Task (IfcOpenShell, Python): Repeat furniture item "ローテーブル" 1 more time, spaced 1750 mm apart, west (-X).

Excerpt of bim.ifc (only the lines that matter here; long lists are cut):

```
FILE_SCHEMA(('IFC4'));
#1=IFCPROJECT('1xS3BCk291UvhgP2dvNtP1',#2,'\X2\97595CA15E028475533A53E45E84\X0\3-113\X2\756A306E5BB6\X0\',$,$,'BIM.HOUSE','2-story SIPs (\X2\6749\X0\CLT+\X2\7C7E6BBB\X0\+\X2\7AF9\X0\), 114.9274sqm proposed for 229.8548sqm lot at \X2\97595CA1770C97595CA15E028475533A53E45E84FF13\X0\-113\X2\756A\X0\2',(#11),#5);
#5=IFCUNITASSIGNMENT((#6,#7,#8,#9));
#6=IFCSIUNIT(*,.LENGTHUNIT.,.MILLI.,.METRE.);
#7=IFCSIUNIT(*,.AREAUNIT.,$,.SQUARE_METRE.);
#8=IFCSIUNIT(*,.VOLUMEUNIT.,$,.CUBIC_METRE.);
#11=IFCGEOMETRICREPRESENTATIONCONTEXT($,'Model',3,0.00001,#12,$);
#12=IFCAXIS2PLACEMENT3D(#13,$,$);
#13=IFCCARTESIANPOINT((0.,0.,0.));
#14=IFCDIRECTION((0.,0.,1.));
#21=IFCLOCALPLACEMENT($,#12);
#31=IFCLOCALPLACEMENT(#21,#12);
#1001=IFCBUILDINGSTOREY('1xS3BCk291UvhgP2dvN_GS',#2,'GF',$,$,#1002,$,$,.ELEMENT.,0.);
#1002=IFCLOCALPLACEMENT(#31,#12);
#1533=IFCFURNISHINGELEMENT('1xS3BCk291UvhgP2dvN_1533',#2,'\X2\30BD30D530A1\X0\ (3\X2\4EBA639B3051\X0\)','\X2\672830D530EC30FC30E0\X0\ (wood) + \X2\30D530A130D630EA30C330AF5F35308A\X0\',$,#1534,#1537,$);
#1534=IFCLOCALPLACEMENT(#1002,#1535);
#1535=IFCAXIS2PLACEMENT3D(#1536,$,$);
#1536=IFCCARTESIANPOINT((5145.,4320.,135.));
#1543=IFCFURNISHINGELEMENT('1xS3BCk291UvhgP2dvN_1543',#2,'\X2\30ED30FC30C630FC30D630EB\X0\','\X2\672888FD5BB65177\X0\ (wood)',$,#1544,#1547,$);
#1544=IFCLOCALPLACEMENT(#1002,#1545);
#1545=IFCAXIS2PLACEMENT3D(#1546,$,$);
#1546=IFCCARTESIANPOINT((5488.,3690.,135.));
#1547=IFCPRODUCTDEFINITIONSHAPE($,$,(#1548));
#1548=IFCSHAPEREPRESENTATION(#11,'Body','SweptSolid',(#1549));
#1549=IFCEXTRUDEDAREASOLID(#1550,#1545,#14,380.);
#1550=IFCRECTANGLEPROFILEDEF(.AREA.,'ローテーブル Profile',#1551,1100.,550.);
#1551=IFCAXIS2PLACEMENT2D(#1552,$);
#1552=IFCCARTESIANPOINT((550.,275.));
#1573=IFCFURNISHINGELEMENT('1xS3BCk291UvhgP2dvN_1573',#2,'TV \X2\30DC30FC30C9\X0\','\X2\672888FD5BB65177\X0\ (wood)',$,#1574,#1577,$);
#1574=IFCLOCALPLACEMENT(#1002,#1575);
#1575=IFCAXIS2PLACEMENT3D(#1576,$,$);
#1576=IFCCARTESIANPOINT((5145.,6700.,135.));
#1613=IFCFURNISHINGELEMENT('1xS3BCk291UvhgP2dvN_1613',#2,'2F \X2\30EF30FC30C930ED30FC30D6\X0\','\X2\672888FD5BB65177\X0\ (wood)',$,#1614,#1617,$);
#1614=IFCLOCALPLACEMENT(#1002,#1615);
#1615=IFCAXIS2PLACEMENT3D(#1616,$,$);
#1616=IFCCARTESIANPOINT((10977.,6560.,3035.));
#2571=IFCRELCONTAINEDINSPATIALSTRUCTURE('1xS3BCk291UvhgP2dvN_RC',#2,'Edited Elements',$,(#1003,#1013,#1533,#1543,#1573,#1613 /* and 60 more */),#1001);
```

```python
import numpy as np
import ifcopenshell
import ifcopenshell.api.geometry
import ifcopenshell.api.root
import ifcopenshell.util.element
import ifcopenshell.util.placement

model = ifcopenshell.open("bim.ifc")


def reuse_history(source, copy):
    """copy_class also copies each property set's owner history, people and application; keep the originals."""
    for rel in copy.IsDefinedBy:
        if rel.is_a("IfcRelDefinesByProperties") and (history := rel.RelatingPropertyDefinition.OwnerHistory):
            rel.RelatingPropertyDefinition.OwnerHistory = source.OwnerHistory
            ifcopenshell.util.element.remove_deep2(model, history)


source = model.by_guid("1xS3BCk291UvhgP2dvN_1543")
base = ifcopenshell.util.placement.get_local_placement(source.ObjectPlacement)
step = np.array([-1.0, 0.0, 0.0]) * 1750.0

for i in range(1, 2):
    copy = ifcopenshell.api.root.copy_class(model, product=source)
    copy.Representation = ifcopenshell.util.element.copy_deep(
        model, source.Representation, exclude=["IfcGeometricRepresentationContext", "IfcRepresentationMap"]
    )
    reuse_history(source, copy)
    matrix = base.copy()
    matrix[:3, 3] += i * step
    print("added at", matrix[:3, 3].round(3) + 0.0)
    ifcopenshell.api.geometry.edit_object_placement(model, product=copy, matrix=matrix, is_si=False)

model.write("bim_updated.ifc")
```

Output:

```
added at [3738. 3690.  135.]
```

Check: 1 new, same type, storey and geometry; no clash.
